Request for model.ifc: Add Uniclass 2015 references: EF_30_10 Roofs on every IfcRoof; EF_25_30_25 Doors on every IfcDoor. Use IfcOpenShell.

First a look at what the model holds.

```python
import ifcopenshell

model = ifcopenshell.open("model.ifc")
print(model.schema)
print("classifications:", [c.Name for c in model.by_type("IfcClassification")])
for ifc_class in ("IfcDoor", "IfcRoof", "IfcStair", "IfcWall", "IfcWindow"):
    print(ifc_class, len(model.by_type(ifc_class)))
```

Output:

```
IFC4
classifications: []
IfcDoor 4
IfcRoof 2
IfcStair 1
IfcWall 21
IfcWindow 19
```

```python
import ifcopenshell
import ifcopenshell.api.classification

model = ifcopenshell.open("model.ifc")

system = ifcopenshell.api.classification.add_classification(model, classification="Uniclass 2015")

codes = {
    "IfcRoof": ("EF_30_10", "Roofs"),
    "IfcDoor": ("EF_25_30_25", "Doors"),
}
for ifc_class, (code, name) in codes.items():
    products = model.by_type(ifc_class)
    ifcopenshell.api.classification.add_reference(
        model, products=products, classification=system, identification=code, name=name
    )
    print(code, len(products))

model.write("model-out.ifc")
```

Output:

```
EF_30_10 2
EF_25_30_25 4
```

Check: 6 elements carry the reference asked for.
